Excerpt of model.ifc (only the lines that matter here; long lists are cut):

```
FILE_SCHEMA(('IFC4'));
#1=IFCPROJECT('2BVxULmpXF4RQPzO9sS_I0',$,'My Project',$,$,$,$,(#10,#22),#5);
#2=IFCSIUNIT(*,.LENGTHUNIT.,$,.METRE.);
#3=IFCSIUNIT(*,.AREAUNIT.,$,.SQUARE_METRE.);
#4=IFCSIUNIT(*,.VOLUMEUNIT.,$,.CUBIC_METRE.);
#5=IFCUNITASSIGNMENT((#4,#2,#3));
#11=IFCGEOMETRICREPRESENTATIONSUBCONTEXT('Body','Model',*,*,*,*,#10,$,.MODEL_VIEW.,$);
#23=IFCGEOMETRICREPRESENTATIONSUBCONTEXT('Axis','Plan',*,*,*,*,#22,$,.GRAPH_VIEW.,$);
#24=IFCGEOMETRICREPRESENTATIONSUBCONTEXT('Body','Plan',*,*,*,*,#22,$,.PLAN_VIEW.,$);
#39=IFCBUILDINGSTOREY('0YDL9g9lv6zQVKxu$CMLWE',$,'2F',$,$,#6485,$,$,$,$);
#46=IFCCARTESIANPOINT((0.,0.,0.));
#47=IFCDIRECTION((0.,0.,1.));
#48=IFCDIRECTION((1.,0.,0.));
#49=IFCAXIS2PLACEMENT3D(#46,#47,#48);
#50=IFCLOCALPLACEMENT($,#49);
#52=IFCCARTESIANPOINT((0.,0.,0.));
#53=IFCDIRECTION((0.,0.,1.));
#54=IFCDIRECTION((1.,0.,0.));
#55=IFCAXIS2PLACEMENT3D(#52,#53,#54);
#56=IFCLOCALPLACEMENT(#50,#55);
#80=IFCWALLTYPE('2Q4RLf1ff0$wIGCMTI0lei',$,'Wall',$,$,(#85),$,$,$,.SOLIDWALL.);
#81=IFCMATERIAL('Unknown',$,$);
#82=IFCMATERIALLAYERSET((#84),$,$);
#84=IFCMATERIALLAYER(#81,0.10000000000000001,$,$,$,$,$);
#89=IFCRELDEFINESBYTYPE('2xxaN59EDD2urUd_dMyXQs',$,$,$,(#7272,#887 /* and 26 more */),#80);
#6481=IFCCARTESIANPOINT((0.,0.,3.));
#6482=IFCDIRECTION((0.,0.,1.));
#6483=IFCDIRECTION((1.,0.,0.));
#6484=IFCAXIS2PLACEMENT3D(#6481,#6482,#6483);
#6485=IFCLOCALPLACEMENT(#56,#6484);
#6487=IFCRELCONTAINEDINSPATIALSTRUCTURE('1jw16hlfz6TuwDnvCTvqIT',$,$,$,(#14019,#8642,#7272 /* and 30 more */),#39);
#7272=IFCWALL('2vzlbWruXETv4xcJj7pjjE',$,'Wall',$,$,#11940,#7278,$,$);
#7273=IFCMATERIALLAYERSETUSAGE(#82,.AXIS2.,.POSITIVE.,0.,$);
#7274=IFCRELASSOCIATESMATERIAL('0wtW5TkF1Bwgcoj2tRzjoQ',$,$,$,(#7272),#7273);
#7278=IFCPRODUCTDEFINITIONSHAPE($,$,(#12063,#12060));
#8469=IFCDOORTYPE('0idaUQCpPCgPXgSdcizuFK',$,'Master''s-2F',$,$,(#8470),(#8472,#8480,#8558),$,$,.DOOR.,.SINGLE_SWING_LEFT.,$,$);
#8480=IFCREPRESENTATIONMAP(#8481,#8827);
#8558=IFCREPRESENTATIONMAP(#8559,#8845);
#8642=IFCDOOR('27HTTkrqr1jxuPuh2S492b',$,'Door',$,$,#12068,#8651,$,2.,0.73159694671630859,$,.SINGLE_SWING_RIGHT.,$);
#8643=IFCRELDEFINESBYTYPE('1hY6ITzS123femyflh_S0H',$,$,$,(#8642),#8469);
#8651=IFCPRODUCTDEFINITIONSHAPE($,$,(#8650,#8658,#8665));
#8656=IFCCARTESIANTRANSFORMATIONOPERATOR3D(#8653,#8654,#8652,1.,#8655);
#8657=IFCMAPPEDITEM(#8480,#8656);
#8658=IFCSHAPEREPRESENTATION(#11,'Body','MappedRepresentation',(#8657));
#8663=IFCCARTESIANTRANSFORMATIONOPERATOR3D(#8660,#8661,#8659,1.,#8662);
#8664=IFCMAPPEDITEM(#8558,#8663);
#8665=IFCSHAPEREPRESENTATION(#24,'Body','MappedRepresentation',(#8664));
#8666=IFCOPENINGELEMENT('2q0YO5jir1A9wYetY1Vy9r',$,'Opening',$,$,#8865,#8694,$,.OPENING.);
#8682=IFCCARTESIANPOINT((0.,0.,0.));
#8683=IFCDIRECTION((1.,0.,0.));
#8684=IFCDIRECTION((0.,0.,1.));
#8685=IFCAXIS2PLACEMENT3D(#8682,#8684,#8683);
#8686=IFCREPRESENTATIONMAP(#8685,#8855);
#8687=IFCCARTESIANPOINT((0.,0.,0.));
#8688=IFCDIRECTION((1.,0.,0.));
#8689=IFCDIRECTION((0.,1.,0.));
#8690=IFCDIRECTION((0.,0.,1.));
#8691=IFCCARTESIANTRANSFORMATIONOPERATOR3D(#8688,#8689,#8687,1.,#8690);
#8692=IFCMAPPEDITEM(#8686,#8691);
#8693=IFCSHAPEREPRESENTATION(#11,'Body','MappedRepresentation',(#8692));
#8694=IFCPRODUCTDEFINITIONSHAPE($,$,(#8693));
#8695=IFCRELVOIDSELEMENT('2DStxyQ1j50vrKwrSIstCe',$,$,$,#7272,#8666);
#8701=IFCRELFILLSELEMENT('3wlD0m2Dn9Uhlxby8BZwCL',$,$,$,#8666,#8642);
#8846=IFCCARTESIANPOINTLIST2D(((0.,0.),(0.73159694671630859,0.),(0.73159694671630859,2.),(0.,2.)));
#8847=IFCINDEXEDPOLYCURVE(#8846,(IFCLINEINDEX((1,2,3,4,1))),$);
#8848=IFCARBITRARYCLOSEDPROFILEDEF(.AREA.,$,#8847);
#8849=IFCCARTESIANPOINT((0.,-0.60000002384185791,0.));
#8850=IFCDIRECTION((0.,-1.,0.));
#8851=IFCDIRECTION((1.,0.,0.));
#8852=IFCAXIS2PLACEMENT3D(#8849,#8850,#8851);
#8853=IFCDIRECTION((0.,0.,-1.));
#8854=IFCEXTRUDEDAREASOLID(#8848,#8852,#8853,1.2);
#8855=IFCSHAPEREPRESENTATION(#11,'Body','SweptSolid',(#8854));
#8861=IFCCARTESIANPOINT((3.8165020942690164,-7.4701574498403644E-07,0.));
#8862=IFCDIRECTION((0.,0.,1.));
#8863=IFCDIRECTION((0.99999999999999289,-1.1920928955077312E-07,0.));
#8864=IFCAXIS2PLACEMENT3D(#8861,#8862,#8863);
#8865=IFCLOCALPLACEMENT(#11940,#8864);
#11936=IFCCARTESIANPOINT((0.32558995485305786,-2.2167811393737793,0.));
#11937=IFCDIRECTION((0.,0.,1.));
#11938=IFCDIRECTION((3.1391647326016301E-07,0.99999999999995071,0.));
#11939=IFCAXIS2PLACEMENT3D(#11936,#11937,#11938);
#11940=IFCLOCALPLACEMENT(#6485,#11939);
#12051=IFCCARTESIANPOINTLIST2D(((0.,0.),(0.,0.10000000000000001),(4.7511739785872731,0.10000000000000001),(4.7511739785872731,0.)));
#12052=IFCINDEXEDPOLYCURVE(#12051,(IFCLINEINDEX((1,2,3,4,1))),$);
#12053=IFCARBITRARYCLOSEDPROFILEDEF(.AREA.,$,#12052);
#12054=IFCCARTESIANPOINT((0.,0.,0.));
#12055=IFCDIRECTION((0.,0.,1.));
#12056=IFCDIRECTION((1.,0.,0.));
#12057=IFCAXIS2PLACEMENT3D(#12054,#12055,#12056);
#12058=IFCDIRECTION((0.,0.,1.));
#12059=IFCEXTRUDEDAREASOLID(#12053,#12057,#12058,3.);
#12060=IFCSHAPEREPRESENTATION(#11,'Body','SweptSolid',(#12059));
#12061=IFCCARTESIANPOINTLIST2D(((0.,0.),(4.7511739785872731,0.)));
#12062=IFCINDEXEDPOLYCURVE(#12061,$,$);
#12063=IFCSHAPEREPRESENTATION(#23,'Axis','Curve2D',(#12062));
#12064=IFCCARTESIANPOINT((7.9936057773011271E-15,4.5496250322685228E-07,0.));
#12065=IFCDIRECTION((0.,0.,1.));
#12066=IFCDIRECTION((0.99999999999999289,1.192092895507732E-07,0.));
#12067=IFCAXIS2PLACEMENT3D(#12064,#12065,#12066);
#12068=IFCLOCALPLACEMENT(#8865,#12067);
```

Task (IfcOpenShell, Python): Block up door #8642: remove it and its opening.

```python
import ifcopenshell
import ifcopenshell.api.feature
import ifcopenshell.api.root
import ifcopenshell.geom
import ifcopenshell.util.shape

model = ifcopenshell.open("model.ifc")
settings = ifcopenshell.geom.settings()


def volume(element):
    """Net volume in cubic metres, openings subtracted."""
    shape = ifcopenshell.geom.create_shape(settings, element)
    return ifcopenshell.util.shape.get_volume(shape.geometry)


door = model.by_guid("27HTTkrqr1jxuPuh2S492b")
opening = door.FillsVoids[0].RelatingOpeningElement
wall = opening.VoidsElements[0].RelatingBuildingElement
before = volume(wall)

ifcopenshell.api.root.remove_product(model, product=door)
ifcopenshell.api.feature.remove_feature(model, feature=opening)

after = volume(wall)

print(f"wall volume {before:.3f} -> {after:.3f} m3")

model.write("model_rev.ifc")
```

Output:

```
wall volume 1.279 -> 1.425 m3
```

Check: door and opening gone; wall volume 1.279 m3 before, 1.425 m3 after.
